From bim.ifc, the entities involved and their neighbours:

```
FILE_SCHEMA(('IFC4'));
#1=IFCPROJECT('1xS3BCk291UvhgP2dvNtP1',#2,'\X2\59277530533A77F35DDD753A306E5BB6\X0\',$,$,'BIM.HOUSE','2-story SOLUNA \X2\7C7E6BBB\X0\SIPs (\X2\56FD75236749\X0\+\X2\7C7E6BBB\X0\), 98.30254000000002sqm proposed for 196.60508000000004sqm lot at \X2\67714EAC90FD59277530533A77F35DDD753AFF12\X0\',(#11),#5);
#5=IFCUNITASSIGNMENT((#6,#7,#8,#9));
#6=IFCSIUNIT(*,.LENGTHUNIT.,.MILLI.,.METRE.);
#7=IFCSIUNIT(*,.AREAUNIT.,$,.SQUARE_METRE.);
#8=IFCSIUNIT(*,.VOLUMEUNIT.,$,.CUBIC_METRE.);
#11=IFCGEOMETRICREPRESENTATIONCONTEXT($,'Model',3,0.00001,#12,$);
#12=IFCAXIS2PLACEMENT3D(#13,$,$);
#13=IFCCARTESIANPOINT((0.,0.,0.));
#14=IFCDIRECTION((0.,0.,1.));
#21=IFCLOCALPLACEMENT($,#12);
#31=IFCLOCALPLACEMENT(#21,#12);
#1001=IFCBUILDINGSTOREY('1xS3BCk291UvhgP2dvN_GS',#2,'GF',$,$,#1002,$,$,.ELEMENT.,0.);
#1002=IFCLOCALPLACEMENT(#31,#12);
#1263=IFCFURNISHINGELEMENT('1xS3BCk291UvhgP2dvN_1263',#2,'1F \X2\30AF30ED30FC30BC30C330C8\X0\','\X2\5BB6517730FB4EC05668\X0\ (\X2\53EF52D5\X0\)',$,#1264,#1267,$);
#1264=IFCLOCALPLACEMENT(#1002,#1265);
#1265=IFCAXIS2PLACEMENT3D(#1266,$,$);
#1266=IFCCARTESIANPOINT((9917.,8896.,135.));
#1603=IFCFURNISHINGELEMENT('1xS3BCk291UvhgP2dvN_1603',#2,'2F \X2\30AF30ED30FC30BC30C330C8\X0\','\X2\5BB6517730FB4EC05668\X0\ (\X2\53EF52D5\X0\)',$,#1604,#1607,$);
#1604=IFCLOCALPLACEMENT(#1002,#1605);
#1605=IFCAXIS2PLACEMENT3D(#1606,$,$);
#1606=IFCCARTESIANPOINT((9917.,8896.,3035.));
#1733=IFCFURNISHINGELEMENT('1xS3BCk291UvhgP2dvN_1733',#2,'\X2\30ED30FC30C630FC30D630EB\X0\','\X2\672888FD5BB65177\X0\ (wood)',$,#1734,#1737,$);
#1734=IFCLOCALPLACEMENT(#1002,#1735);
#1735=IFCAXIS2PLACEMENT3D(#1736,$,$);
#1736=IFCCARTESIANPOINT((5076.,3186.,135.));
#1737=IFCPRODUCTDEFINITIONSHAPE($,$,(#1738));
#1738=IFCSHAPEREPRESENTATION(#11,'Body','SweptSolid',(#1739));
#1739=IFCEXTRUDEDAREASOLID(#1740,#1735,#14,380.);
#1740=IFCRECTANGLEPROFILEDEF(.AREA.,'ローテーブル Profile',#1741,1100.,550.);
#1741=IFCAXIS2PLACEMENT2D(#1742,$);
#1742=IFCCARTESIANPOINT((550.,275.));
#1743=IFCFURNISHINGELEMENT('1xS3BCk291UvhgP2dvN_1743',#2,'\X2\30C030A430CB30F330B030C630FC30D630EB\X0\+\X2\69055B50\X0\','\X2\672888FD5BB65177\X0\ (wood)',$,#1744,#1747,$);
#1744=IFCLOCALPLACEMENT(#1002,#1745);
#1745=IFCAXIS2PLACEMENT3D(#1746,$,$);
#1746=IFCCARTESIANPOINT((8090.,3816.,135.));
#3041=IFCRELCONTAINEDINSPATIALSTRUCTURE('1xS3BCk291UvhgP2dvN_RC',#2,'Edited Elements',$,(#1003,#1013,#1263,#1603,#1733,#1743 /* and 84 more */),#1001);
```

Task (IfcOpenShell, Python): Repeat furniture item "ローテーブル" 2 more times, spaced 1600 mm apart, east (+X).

```python
import numpy as np
import ifcopenshell
import ifcopenshell.api.geometry
import ifcopenshell.api.root
import ifcopenshell.util.element
import ifcopenshell.util.placement
import ifcopenshell.util.unit

model = ifcopenshell.open("bim.ifc")
unit_scale = ifcopenshell.util.unit.calculate_unit_scale(model)


def reuse_history(source, copy):
    """copy_class also copies each property set's owner history, people and application; keep the originals."""
    for rel in copy.IsDefinedBy:
        if rel.is_a("IfcRelDefinesByProperties") and (history := rel.RelatingPropertyDefinition.OwnerHistory):
            rel.RelatingPropertyDefinition.OwnerHistory = source.OwnerHistory
            ifcopenshell.util.element.remove_deep2(model, history)


source = model.by_guid("1xS3BCk291UvhgP2dvN_1733")
base = ifcopenshell.util.placement.get_local_placement(source.ObjectPlacement)
step = np.array([1.0, 0.0, 0.0]) * 1.6 / unit_scale

for i in range(1, 3):
    copy = ifcopenshell.api.root.copy_class(model, product=source)
    copy.Representation = ifcopenshell.util.element.copy_deep(
        model, source.Representation, exclude=["IfcGeometricRepresentationContext", "IfcRepresentationMap"]
    )
    reuse_history(source, copy)
    matrix = base.copy()
    matrix[:3, 3] += i * step
    print("added at", matrix[:3, 3].round(3) + 0.0)
    ifcopenshell.api.geometry.edit_object_placement(model, product=copy, matrix=matrix, is_si=False)

model.write("bim-out.ifc")
```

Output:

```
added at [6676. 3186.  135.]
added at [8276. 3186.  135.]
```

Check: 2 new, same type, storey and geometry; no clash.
